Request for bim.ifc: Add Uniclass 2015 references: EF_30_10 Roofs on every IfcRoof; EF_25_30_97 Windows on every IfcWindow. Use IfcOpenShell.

First a look at what the model holds.

```python
import ifcopenshell

model = ifcopenshell.open("bim.ifc")
print(model.schema)
print("classifications:", [c.Name for c in model.by_type("IfcClassification")])
for ifc_class in ("IfcDoor", "IfcRoof", "IfcStair", "IfcWall", "IfcWindow"):
    print(ifc_class, len(model.by_type(ifc_class)))
```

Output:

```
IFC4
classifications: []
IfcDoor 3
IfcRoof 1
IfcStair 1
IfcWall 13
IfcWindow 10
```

```python
import ifcopenshell
import ifcopenshell.api.classification

model = ifcopenshell.open("bim.ifc")

system = ifcopenshell.api.classification.add_classification(model, classification="Uniclass 2015")

codes = {
    "IfcRoof": ("EF_30_10", "Roofs"),
    "IfcWindow": ("EF_25_30_97", "Windows"),
}
for ifc_class, (code, name) in codes.items():
    products = model.by_type(ifc_class)
    ifcopenshell.api.classification.add_reference(
        model, products=products, classification=system, identification=code, name=name
    )
    print(code, len(products))

model.write("bim_edited.ifc")
```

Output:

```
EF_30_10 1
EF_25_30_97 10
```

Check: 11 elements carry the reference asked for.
